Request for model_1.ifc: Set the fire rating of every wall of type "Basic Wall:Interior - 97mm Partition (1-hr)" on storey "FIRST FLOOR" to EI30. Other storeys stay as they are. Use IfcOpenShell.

First a look at what the model holds.

```python
import ifcopenshell
import ifcopenshell.util.element

model = ifcopenshell.open("model_1.ifc")
print(model.schema)
storey = next(s for s in model.by_type("IfcBuildingStorey") if s.Name == "FIRST FLOOR")
walls = [e for e in ifcopenshell.util.element.get_decomposition(storey) if e.is_a("IfcWall")]
seen = {}
for e in walls:
    element_type = ifcopenshell.util.element.get_type(e)
    key = (element_type.Name if element_type != e and element_type else None, ifcopenshell.util.element.get_pset(e, "Pset_WallCommon", "FireRating"))
    seen[key] = seen.get(key, 0) + 1
for (name, value), count in sorted(seen.items(), key=str):
    print(count, "x", name, "|", value)
```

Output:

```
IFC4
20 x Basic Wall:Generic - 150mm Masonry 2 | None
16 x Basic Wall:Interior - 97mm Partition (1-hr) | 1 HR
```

```python
import ifcopenshell
import ifcopenshell.api.pset
import ifcopenshell.util.element

model = ifcopenshell.open("model_1.ifc")

storey = next(s for s in model.by_type("IfcBuildingStorey") if s.Name == "FIRST FLOOR")
walls = [e for e in ifcopenshell.util.element.get_decomposition(storey) if e.is_a("IfcWall")]

count = 0
for e in walls:
    element_type = ifcopenshell.util.element.get_type(e)
    if element_type in (None, e) or element_type.Name != "Basic Wall:Interior - 97mm Partition (1-hr)":
        continue
    # add_pset returns the element's existing set when there is one.
    pset = ifcopenshell.api.pset.add_pset(model, product=e, name="Pset_WallCommon")
    ifcopenshell.api.pset.edit_pset(model, pset=pset, properties={"FireRating": "EI30"})
    count += 1

print(count, "walls updated")

model.write("model_1_rev.ifc")
```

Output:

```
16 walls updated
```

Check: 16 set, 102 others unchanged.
